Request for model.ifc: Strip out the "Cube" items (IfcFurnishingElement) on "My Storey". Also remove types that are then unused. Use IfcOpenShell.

First a look at what the model holds.

```python
import ifcopenshell
import ifcopenshell.util.element

model = ifcopenshell.open("model.ifc")
print(model.schema)
storey = next(s for s in model.by_type("IfcBuildingStorey") if s.Name == "My Storey")
furniture = [e for e in ifcopenshell.util.element.get_decomposition(storey) if e.is_a("IfcFurnishingElement")]
seen = {}
for e in furniture:
    element_type = ifcopenshell.util.element.get_type(e)
    name = element_type.Name if element_type not in (None, e) else None
    seen[name] = seen.get(name, 0) + 1
for name, count in sorted(seen.items(), key=str):
    print(count, "x", name)
```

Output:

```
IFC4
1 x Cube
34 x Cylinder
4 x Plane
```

```python
import ifcopenshell
import ifcopenshell.api.root
import ifcopenshell.util.element

model = ifcopenshell.open("model.ifc")

storey = next(s for s in model.by_type("IfcBuildingStorey") if s.Name == "My Storey")
furniture = [e for e in ifcopenshell.util.element.get_decomposition(storey) if e.is_a("IfcFurnishingElement")]
targets = [e for e in furniture if (t := ifcopenshell.util.element.get_type(e)) not in (None, e) and t.Name == "Cube"]
types = {ifcopenshell.util.element.get_type(e) for e in targets} - {None, *targets}

for e in targets:
    ifcopenshell.api.root.remove_product(model, product=e)
print(len(targets), "removed")

unused = [t for t in types if not ifcopenshell.util.element.get_types(t)]
for t in unused:
    ifcopenshell.api.root.remove_product(model, product=t)
print(len(unused), "unused types removed")

model.write("model_updated.ifc")
```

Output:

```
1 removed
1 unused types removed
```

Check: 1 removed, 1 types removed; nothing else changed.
